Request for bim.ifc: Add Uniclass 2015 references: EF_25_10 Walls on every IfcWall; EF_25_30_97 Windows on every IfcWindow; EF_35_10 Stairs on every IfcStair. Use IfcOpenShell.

First a look at what the model holds.

```python
import ifcopenshell

model = ifcopenshell.open("bim.ifc")
print(model.schema)
print("classifications:", [c.Name for c in model.by_type("IfcClassification")])
for ifc_class in ("IfcDoor", "IfcRoof", "IfcStair", "IfcWall", "IfcWindow"):
    print(ifc_class, len(model.by_type(ifc_class)))
```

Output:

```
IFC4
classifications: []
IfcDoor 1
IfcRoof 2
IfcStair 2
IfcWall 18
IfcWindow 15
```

```python
import ifcopenshell
import ifcopenshell.api.classification

model = ifcopenshell.open("bim.ifc")

system = ifcopenshell.api.classification.add_classification(model, classification="Uniclass 2015")

codes = {
    "IfcWall": ("EF_25_10", "Walls"),
    "IfcWindow": ("EF_25_30_97", "Windows"),
    "IfcStair": ("EF_35_10", "Stairs"),
}
for ifc_class, (code, name) in codes.items():
    products = model.by_type(ifc_class)
    ifcopenshell.api.classification.add_reference(
        model, products=products, classification=system, identification=code, name=name
    )
    print(code, len(products))

model.write("bim_updated.ifc")
```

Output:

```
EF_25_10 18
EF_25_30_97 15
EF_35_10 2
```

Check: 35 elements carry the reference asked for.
